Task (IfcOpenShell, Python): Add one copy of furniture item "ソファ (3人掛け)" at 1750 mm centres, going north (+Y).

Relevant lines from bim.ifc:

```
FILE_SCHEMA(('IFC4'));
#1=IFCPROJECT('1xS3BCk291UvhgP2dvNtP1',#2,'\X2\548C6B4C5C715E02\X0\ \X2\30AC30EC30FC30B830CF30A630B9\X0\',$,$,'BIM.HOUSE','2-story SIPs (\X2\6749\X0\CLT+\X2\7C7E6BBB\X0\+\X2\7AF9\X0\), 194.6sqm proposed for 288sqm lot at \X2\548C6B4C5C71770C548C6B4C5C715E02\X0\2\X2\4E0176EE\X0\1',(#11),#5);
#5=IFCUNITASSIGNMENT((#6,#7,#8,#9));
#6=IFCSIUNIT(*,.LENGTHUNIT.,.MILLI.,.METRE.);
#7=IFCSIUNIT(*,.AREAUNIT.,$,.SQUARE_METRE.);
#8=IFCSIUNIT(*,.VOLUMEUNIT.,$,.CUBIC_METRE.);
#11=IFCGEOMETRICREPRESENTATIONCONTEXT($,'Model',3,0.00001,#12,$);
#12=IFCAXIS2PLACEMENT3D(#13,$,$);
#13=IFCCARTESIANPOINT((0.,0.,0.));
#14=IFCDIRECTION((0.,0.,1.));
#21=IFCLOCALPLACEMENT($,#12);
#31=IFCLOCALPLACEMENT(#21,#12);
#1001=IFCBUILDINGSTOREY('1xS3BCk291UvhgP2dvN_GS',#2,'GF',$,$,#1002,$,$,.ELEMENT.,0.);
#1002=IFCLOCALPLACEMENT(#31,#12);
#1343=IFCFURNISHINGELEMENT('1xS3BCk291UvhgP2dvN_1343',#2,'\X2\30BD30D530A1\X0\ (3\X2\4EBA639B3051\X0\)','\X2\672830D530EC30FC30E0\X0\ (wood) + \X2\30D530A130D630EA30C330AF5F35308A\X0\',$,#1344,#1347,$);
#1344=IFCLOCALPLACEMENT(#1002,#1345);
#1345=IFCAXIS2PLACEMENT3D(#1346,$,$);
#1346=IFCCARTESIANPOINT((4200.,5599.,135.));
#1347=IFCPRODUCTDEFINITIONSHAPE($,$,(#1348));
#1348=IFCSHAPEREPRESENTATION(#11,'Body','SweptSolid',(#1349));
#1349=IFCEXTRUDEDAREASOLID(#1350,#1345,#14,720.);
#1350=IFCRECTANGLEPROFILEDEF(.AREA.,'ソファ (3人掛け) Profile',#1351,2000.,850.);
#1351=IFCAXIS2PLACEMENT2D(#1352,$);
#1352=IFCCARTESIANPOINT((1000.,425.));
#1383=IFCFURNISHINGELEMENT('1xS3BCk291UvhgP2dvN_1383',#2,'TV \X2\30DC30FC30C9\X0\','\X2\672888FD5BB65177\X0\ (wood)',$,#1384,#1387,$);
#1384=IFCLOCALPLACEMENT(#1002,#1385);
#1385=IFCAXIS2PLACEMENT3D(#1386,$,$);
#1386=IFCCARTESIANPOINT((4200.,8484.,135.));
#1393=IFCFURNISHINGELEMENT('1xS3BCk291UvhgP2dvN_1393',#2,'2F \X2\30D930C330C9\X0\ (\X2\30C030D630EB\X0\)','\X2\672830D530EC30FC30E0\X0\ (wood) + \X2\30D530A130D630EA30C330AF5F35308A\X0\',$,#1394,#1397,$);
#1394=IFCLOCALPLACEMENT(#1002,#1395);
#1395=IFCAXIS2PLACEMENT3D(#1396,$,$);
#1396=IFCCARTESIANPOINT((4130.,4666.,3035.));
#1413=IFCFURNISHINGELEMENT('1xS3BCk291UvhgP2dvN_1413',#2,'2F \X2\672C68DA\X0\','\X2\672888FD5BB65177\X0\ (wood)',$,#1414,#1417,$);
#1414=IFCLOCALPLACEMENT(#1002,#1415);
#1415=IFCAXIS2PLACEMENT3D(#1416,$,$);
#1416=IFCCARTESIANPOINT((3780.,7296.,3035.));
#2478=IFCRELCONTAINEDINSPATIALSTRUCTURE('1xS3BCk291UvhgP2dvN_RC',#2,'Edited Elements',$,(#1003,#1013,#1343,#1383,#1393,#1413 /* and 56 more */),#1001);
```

```python
import numpy as np
import ifcopenshell
import ifcopenshell.api.geometry
import ifcopenshell.api.root
import ifcopenshell.util.element
import ifcopenshell.util.placement
import ifcopenshell.util.unit

model = ifcopenshell.open("bim.ifc")
unit_scale = ifcopenshell.util.unit.calculate_unit_scale(model)


def reuse_history(source, copy):
    """copy_class also copies each property set's owner history, people and application; keep the originals."""
    for rel in copy.IsDefinedBy:
        if rel.is_a("IfcRelDefinesByProperties") and (history := rel.RelatingPropertyDefinition.OwnerHistory):
            rel.RelatingPropertyDefinition.OwnerHistory = source.OwnerHistory
            ifcopenshell.util.element.remove_deep2(model, history)


source = model.by_guid("1xS3BCk291UvhgP2dvN_1343")
base = ifcopenshell.util.placement.get_local_placement(source.ObjectPlacement)
step = np.array([0.0, 1.0, 0.0]) * 1.75 / unit_scale

for i in range(1, 2):
    copy = ifcopenshell.api.root.copy_class(model, product=source)
    copy.Representation = ifcopenshell.util.element.copy_deep(
        model, source.Representation, exclude=["IfcGeometricRepresentationContext", "IfcRepresentationMap"]
    )
    reuse_history(source, copy)
    matrix = base.copy()
    matrix[:3, 3] += i * step
    print("added at", matrix[:3, 3].round(3) + 0.0)
    ifcopenshell.api.geometry.edit_object_placement(model, product=copy, matrix=matrix, is_si=False)

model.write("bim-out.ifc")
```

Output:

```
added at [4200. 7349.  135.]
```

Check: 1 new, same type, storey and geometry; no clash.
